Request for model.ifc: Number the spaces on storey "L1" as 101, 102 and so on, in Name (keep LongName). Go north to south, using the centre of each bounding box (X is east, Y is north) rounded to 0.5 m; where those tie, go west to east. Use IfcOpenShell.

First a look at what the model holds.

```python
import ifcopenshell
import ifcopenshell.util.element
import ifcopenshell.util.placement

model = ifcopenshell.open("model.ifc")
print(model.schema)
storey = next(s for s in model.by_type("IfcBuildingStorey") if s.Name == "L1")
spaces = [e for e in ifcopenshell.util.element.get_decomposition(storey) if e.is_a("IfcSpace")]
for e in sorted(spaces, key=lambda e: e.id()):
    origin = ifcopenshell.util.placement.get_local_placement(e.ObjectPlacement)[:3, 3]
    print(e.id(), e.Name, e.LongName, origin.round(2) + 0.0, sep=" | ")
```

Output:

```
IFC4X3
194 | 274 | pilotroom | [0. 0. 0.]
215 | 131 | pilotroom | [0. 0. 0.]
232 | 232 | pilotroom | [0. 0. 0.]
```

```python
import ifcopenshell
import ifcopenshell.geom
import ifcopenshell.util.element
import ifcopenshell.util.shape

model = ifcopenshell.open("model.ifc")
settings = ifcopenshell.geom.settings()
settings.set("use-world-coords", True)


def centre(element):
    shape = ifcopenshell.geom.create_shape(settings, element)
    return ifcopenshell.util.shape.get_bbox_centroid(shape.geometry)


storey = next(s for s in model.by_type("IfcBuildingStorey") if s.Name == "L1")
spaces = [e for e in ifcopenshell.util.element.get_decomposition(storey) if e.is_a("IfcSpace")]

# Insertion points can sit at a corner or the storey origin, so sort by the geometry (in metres).
centres = {e: centre(e) for e in spaces}
spaces.sort(key=lambda e: (-round(centres[e][1] / 0.5), centres[e][0]))

for i, e in enumerate(spaces, start=1):
    number = f"1{i:02d}"
    e.Name = number
    print(e.id(), number)

model.write("model_rev.ifc")
```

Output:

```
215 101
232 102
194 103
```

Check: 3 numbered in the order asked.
